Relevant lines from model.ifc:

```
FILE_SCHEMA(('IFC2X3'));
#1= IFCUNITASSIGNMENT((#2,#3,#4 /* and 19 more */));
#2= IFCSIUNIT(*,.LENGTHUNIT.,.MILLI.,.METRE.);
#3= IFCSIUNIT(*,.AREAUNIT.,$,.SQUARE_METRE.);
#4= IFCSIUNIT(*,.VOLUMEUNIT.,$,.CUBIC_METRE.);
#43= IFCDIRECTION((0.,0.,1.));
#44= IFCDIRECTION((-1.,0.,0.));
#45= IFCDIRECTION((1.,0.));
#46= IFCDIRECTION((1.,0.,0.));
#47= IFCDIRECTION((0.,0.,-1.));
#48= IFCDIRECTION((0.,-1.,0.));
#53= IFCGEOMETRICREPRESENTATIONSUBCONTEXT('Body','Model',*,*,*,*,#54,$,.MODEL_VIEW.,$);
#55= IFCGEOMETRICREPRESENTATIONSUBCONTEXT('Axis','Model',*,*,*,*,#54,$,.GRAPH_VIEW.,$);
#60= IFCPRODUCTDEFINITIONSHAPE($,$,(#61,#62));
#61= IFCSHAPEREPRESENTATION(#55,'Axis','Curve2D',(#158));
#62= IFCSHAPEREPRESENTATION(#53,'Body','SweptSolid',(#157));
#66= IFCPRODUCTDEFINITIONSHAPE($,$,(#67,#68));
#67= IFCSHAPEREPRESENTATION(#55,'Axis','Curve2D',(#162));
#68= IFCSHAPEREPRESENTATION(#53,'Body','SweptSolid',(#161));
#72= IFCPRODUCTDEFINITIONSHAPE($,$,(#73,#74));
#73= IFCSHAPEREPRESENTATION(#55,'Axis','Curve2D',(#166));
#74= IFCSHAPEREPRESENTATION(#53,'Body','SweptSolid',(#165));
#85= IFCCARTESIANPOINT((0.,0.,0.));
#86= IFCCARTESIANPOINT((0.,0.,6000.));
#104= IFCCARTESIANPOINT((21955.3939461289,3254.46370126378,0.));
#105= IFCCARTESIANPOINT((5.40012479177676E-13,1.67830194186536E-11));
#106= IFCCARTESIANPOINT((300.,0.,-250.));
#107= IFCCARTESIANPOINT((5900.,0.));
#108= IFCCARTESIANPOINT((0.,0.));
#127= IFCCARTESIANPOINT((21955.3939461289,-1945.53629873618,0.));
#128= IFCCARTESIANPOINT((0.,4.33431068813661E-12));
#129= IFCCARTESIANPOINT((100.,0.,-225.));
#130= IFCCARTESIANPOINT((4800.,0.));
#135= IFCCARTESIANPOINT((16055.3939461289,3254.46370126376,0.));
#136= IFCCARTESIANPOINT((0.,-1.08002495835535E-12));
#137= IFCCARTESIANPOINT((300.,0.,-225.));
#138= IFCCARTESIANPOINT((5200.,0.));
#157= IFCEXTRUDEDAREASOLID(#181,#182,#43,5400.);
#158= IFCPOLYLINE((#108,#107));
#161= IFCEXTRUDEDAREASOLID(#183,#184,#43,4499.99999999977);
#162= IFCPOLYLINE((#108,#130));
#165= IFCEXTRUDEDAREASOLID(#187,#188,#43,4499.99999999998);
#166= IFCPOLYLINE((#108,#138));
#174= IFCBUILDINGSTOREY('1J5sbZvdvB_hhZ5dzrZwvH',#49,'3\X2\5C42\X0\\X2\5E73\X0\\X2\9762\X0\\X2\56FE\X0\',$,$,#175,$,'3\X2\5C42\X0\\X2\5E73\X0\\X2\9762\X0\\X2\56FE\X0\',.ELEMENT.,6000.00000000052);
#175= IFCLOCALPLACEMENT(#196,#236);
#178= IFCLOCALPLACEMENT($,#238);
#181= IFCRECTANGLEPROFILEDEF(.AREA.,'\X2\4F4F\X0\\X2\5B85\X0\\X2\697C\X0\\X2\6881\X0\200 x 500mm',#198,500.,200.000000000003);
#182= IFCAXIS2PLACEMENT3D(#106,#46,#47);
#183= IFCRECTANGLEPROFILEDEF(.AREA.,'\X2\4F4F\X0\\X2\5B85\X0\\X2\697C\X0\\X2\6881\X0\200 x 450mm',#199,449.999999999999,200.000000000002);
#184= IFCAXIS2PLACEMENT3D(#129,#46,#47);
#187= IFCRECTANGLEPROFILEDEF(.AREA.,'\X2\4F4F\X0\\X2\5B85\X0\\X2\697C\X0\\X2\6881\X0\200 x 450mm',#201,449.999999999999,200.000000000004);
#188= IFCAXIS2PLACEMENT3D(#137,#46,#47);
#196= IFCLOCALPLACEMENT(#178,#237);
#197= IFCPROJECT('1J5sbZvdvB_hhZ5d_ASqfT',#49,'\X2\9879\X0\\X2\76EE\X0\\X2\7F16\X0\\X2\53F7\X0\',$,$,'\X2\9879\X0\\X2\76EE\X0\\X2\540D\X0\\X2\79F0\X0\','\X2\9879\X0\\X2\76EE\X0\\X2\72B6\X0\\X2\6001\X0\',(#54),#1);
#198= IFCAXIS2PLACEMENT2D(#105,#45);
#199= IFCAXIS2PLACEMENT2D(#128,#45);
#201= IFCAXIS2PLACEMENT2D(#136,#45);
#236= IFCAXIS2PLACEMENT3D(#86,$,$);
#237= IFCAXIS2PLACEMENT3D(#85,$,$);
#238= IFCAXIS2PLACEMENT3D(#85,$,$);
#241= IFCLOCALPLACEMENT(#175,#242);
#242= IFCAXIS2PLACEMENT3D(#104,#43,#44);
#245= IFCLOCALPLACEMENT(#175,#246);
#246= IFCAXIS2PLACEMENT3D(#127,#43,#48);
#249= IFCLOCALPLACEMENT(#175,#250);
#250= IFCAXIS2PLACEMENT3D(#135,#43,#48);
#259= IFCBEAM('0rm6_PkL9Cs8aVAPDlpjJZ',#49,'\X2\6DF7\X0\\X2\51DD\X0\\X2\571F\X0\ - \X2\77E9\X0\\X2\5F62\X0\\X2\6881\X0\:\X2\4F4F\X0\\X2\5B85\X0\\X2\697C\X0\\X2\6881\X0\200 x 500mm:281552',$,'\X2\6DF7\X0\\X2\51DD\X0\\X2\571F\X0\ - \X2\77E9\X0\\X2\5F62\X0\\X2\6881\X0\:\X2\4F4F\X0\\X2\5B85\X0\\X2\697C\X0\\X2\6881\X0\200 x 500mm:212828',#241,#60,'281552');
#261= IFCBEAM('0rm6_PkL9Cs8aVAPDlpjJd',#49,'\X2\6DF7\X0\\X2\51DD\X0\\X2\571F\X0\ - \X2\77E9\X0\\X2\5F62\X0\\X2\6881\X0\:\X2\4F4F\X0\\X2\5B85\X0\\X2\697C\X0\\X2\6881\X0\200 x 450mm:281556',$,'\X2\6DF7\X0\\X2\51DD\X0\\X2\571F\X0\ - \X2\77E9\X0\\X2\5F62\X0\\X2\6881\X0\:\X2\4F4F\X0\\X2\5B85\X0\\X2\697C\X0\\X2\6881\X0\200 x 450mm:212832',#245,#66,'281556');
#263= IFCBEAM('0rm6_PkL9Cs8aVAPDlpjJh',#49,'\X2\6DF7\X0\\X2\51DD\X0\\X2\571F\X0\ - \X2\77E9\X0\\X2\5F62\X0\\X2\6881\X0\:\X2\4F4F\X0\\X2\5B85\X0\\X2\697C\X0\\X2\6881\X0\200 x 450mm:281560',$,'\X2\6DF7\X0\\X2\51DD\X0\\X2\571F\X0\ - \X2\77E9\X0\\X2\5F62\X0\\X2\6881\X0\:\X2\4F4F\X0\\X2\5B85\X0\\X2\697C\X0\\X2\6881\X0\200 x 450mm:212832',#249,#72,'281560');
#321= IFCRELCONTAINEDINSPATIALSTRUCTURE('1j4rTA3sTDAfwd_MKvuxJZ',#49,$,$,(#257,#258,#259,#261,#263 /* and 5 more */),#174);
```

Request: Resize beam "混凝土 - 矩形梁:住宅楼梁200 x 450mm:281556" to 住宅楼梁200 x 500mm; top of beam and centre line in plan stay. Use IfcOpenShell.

```python
import ifcopenshell
import ifcopenshell.util.element
import ifcopenshell.util.representation

model = ifcopenshell.open("model.ifc")

member = model.by_id(261)
source = next(p for p in model.by_type("IfcRectangleProfileDef") if p.ProfileName == "住宅楼梁200 x 500mm")

body = ifcopenshell.util.representation.get_representation(member, "Model", "Body")
solid = body.Items[0]
old_profile = solid.SweptArea

# Copy the section's sizes but keep this member's own profile position.
profile = ifcopenshell.util.element.copy(model, source)
# Profiles are centred, so shift by half the change in depth to hold the top.
shift = (old_profile.XDim - profile.XDim) / 2
x, y = old_profile.Position.Location.Coordinates
up = (-1.0, 0.0)  # upwards, in the solid's own plane
location = model.createIfcCartesianPoint((x + up[0] * shift, y + up[1] * shift))
profile.Position = model.createIfcAxis2Placement2D(location, old_profile.Position.RefDirection)
solid.SweptArea = profile
if not model.get_total_inverses(old_profile):
    ifcopenshell.util.element.remove_deep2(model, old_profile)
member.Name = member.Name.replace("住宅楼梁200 x 450mm", "住宅楼梁200 x 500mm")
member.ObjectType = member.ObjectType.replace("住宅楼梁200 x 450mm", "住宅楼梁200 x 500mm")

print(solid.SweptArea)

model.write("model_v2.ifc")
```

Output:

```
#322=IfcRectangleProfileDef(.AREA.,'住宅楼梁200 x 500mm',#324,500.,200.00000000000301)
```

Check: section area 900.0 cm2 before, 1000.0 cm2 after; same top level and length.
